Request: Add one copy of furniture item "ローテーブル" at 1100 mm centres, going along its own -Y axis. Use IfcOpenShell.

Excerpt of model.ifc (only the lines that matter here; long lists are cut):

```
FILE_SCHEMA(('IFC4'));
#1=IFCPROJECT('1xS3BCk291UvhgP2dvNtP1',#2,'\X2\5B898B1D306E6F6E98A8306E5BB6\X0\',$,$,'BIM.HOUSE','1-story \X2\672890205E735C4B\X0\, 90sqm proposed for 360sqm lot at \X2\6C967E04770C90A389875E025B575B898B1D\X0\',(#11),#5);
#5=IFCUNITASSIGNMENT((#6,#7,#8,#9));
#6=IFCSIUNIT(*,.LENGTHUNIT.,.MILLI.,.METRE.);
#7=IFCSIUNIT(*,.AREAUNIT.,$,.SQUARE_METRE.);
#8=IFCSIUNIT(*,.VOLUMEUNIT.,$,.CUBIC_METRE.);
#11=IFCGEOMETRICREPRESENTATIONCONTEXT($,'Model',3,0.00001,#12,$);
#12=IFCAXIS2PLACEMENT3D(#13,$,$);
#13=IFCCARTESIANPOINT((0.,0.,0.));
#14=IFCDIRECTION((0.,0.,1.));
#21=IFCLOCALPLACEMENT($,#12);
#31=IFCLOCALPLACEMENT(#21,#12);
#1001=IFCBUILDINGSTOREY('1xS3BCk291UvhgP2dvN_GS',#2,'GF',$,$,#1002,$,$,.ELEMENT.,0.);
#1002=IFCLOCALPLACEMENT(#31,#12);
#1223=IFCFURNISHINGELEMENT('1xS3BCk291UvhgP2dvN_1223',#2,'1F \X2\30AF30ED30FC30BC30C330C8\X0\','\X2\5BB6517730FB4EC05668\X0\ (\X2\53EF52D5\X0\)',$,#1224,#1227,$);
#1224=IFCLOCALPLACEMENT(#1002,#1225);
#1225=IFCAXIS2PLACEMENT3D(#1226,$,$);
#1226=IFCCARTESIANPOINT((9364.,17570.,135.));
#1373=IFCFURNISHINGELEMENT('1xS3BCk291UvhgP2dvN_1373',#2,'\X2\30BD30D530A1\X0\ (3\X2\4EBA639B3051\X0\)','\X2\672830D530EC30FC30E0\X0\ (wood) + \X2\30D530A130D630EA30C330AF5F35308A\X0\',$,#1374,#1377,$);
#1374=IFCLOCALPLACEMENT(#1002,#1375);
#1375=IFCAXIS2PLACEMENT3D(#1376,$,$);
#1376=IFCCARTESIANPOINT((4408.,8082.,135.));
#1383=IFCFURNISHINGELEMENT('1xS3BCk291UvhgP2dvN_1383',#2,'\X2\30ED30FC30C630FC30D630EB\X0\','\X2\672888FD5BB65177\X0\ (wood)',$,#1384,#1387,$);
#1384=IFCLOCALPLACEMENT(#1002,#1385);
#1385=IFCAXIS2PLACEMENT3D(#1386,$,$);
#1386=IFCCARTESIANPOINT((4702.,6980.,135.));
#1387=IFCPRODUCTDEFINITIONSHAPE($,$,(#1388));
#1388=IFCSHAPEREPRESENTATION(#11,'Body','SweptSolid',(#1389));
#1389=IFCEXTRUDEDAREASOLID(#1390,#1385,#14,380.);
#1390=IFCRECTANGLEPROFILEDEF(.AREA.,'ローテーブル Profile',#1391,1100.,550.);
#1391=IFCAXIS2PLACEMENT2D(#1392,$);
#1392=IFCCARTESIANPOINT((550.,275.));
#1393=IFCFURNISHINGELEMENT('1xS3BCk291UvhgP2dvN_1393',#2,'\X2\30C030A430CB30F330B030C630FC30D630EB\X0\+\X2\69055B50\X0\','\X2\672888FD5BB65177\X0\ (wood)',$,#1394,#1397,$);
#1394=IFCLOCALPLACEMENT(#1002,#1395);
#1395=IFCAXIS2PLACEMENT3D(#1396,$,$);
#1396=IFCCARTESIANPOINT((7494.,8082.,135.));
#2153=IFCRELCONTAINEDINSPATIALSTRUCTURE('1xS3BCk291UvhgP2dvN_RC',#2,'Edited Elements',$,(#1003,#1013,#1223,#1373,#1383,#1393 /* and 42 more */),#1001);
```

```python
import ifcopenshell
import ifcopenshell.api.geometry
import ifcopenshell.api.root
import ifcopenshell.util.element
import ifcopenshell.util.placement

model = ifcopenshell.open("model.ifc")


def reuse_history(source, copy):
    """copy_class also copies each property set's owner history, people and application; keep the originals."""
    for rel in copy.IsDefinedBy:
        if rel.is_a("IfcRelDefinesByProperties") and (history := rel.RelatingPropertyDefinition.OwnerHistory):
            rel.RelatingPropertyDefinition.OwnerHistory = source.OwnerHistory
            ifcopenshell.util.element.remove_deep2(model, history)


source = model.by_guid("1xS3BCk291UvhgP2dvN_1383")
base = ifcopenshell.util.placement.get_local_placement(source.ObjectPlacement)
step = -base[:3, 1] * 1100.0

for i in range(1, 2):
    copy = ifcopenshell.api.root.copy_class(model, product=source)
    copy.Representation = ifcopenshell.util.element.copy_deep(
        model, source.Representation, exclude=["IfcGeometricRepresentationContext", "IfcRepresentationMap"]
    )
    reuse_history(source, copy)
    matrix = base.copy()
    matrix[:3, 3] += i * step
    print("added at", matrix[:3, 3].round(3) + 0.0)
    ifcopenshell.api.geometry.edit_object_placement(model, product=copy, matrix=matrix, is_si=False)

model.write("model_v2.ifc")
```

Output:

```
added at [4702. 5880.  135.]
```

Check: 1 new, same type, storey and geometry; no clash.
